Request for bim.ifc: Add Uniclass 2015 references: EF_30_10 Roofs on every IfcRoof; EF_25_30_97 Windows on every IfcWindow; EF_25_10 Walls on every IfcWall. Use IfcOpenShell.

First a look at what the model holds.

```python
import ifcopenshell

model = ifcopenshell.open("bim.ifc")
print(model.schema)
print("classifications:", [c.Name for c in model.by_type("IfcClassification")])
for ifc_class in ("IfcDoor", "IfcRoof", "IfcStair", "IfcWall", "IfcWindow"):
    print(ifc_class, len(model.by_type(ifc_class)))
```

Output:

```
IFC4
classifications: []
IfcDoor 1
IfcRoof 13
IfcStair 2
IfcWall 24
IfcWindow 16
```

```python
import ifcopenshell
import ifcopenshell.api.classification

model = ifcopenshell.open("bim.ifc")

system = ifcopenshell.api.classification.add_classification(model, classification="Uniclass 2015")

codes = {
    "IfcRoof": ("EF_30_10", "Roofs"),
    "IfcWindow": ("EF_25_30_97", "Windows"),
    "IfcWall": ("EF_25_10", "Walls"),
}
for ifc_class, (code, name) in codes.items():
    products = model.by_type(ifc_class)
    ifcopenshell.api.classification.add_reference(
        model, products=products, classification=system, identification=code, name=name
    )
    print(code, len(products))

model.write("bim_v2.ifc")
```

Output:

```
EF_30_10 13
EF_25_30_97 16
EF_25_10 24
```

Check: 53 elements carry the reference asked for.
